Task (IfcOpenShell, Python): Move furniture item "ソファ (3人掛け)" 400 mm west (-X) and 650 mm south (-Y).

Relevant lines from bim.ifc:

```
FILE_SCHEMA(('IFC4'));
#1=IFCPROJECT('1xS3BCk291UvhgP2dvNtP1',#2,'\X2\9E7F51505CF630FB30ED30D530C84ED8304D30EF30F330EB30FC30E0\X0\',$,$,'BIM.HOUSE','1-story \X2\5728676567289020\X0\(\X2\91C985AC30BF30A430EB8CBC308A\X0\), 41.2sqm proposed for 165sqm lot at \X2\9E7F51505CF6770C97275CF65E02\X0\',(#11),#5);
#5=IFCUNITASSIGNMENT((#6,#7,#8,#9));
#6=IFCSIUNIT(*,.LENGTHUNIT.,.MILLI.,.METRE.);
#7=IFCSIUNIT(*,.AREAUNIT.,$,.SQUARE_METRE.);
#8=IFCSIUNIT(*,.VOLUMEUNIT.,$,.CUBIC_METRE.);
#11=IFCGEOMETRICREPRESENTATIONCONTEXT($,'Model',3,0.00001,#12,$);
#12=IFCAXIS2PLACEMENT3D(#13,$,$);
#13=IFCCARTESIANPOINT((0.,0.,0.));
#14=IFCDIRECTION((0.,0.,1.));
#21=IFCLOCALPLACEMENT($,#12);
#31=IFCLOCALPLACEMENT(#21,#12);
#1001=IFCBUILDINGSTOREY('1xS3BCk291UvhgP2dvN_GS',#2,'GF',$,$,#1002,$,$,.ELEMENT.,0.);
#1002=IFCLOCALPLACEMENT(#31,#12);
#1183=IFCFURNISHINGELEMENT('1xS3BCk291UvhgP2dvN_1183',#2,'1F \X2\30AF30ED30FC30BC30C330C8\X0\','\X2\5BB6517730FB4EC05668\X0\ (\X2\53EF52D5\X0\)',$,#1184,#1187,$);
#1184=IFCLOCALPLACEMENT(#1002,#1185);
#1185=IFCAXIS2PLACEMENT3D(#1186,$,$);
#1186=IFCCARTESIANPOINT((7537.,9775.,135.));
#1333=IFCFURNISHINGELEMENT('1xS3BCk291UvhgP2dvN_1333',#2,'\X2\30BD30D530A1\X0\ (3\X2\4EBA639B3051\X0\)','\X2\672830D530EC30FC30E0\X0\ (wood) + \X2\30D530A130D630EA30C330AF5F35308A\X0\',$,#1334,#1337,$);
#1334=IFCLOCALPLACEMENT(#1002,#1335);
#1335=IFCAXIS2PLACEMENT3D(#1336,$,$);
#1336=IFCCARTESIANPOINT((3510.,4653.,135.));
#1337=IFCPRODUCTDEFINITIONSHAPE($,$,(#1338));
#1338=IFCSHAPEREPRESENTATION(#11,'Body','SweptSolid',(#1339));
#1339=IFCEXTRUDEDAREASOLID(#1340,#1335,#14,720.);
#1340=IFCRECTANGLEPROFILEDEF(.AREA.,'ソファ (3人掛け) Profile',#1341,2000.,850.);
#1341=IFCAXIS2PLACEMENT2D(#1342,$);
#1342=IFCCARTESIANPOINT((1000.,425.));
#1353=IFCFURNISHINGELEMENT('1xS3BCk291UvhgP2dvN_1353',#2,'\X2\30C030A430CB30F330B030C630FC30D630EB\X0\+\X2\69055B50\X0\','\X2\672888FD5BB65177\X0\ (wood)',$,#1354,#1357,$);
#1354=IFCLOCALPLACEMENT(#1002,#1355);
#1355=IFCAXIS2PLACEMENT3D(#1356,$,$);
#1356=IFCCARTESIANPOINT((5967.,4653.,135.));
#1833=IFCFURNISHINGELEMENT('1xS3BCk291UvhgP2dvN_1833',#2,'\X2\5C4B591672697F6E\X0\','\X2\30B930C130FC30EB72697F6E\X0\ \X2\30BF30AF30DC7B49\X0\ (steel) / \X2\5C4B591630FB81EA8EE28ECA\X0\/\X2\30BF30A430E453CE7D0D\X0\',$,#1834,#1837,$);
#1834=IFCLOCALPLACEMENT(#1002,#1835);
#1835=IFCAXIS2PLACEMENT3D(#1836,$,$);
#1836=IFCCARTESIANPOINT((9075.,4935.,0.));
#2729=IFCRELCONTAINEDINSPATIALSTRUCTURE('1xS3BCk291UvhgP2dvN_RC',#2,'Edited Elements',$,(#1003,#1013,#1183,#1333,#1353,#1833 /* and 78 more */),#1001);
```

```python
import ifcopenshell
import ifcopenshell.api.geometry
import ifcopenshell.util.placement
import ifcopenshell.util.unit

model = ifcopenshell.open("bim.ifc")
unit_scale = ifcopenshell.util.unit.calculate_unit_scale(model)

item = model.by_guid("1xS3BCk291UvhgP2dvN_1333")
matrix = ifcopenshell.util.placement.get_local_placement(item.ObjectPlacement)
matrix[0, 3] -= 0.4 / unit_scale
matrix[1, 3] -= 0.65 / unit_scale
ifcopenshell.api.geometry.edit_object_placement(model, product=item, matrix=matrix, is_si=False)

print(ifcopenshell.util.placement.get_local_placement(item.ObjectPlacement).round(3) + 0.0)

model.write("bim_updated.ifc")
```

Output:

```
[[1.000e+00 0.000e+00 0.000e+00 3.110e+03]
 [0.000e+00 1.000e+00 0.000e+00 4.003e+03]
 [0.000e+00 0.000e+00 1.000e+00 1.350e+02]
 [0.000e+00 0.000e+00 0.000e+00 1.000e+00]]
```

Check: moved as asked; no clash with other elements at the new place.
